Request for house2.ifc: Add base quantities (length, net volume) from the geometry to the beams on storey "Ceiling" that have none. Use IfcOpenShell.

First a look at what the model holds.

```python
import ifcopenshell
import ifcopenshell.util.element
import ifcopenshell.util.unit

model = ifcopenshell.open("house2.ifc")
print(model.schema)
for unit_type in ("LENGTHUNIT", "AREAUNIT", "VOLUMEUNIT"):
    print(unit_type, ifcopenshell.util.unit.calculate_unit_scale(model, unit_type))
storey = next(s for s in model.by_type("IfcBuildingStorey") if s.Name == "Ceiling")
beams = [e for e in ifcopenshell.util.element.get_decomposition(storey) if e.is_a("IfcBeam")]
for e in sorted(beams, key=lambda e: e.id()):
    print(e.id(), e.is_a(), e.Name, list(ifcopenshell.util.element.get_psets(e, qtos_only=True)), sep=" | ")
```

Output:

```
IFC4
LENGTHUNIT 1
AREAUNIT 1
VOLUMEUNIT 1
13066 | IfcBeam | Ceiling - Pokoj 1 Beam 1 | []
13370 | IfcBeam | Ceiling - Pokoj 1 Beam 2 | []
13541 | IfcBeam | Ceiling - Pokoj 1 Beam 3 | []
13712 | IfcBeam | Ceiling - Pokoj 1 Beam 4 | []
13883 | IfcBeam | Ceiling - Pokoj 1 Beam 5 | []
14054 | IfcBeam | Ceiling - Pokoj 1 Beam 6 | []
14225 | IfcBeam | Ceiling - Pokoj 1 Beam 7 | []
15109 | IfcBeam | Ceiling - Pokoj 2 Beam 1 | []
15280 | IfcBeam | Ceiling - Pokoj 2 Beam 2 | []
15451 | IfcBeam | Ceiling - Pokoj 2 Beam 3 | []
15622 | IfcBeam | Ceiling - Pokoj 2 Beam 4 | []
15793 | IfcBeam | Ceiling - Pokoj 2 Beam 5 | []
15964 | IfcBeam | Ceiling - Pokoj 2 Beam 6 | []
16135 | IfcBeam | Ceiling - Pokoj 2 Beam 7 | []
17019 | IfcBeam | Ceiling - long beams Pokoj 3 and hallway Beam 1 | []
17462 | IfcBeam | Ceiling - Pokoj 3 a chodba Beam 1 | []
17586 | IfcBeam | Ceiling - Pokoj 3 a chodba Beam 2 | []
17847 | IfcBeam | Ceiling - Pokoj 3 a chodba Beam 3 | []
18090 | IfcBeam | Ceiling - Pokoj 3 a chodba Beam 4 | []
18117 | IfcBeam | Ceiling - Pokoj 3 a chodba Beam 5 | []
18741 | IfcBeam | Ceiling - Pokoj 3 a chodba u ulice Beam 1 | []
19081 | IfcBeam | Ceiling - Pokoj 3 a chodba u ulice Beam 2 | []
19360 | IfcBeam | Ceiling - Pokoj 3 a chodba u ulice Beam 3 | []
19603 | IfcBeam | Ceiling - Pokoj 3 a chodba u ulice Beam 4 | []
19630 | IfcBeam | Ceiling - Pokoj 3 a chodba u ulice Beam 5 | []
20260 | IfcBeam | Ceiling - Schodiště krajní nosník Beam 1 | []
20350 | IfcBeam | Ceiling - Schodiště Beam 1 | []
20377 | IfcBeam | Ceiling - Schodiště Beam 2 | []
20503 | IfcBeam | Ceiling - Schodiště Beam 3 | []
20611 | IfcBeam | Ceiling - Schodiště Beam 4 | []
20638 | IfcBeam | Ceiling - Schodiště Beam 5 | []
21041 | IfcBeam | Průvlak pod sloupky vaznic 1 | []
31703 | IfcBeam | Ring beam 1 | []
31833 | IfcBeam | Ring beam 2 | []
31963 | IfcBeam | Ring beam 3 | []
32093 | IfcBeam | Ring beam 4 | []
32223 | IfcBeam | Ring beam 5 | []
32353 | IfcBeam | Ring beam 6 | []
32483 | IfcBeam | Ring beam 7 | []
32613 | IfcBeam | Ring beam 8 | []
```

```python
import ifcopenshell
import ifcopenshell.api.pset
import ifcopenshell.geom
import ifcopenshell.util.element
import ifcopenshell.util.shape
import ifcopenshell.util.unit

model = ifcopenshell.open("house2.ifc")
unit_scale = ifcopenshell.util.unit.calculate_unit_scale(model)
volume_scale = ifcopenshell.util.unit.calculate_unit_scale(model, "VOLUMEUNIT")
settings = ifcopenshell.geom.settings()

storey = next(s for s in model.by_type("IfcBuildingStorey") if s.Name == "Ceiling")
beams = [e for e in ifcopenshell.util.element.get_decomposition(storey) if e.is_a("IfcBeam")]

for e in sorted(beams, key=lambda e: e.id()):
    if ifcopenshell.util.element.get_psets(e, qtos_only=True, should_inherit=False):
        continue
    # Geometry comes back in metres, in the element's own axes.
    shape = ifcopenshell.geom.create_shape(settings, e)
    values = {
        "Length": ifcopenshell.util.shape.get_max_xyz(shape.geometry) / unit_scale,
        "NetVolume": ifcopenshell.util.shape.get_volume(shape.geometry) / volume_scale,
    }
    qto = ifcopenshell.api.pset.add_qto(model, product=e, name="Qto_BeamBaseQuantities")
    ifcopenshell.api.pset.edit_qto(model, qto=qto, properties=values)
    print(e.id(), {k: round(v, 3) for k, v in values.items()})

model.write("house2_updated.ifc")
```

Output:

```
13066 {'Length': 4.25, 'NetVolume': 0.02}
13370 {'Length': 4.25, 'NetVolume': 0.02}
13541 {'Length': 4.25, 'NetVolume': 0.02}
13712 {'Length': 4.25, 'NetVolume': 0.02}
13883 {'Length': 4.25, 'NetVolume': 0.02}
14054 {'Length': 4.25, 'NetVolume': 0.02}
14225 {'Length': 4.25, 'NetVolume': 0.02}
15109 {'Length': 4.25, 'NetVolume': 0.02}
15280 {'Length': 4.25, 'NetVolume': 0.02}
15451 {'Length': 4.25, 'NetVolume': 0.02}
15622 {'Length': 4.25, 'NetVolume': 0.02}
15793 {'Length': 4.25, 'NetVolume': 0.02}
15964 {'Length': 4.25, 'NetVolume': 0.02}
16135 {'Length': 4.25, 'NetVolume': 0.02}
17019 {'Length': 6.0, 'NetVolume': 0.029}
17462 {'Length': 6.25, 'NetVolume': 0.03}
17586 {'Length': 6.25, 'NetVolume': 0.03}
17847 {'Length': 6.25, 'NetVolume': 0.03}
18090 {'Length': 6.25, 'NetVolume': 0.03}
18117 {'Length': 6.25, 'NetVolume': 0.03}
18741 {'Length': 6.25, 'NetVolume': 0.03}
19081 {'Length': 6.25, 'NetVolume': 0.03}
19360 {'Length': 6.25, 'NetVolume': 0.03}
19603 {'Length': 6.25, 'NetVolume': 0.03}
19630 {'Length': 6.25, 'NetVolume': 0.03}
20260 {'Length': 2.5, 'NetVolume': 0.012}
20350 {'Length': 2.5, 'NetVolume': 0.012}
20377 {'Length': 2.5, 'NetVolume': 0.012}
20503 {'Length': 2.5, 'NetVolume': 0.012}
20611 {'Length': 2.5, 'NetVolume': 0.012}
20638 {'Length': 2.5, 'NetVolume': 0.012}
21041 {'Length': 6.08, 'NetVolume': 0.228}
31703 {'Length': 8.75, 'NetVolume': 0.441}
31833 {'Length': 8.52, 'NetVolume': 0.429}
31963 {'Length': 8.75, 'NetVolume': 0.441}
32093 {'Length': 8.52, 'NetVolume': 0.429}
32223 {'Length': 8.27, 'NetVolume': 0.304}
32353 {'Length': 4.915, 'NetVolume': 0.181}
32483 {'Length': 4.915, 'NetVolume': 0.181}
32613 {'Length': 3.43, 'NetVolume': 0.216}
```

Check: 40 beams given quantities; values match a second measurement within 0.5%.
